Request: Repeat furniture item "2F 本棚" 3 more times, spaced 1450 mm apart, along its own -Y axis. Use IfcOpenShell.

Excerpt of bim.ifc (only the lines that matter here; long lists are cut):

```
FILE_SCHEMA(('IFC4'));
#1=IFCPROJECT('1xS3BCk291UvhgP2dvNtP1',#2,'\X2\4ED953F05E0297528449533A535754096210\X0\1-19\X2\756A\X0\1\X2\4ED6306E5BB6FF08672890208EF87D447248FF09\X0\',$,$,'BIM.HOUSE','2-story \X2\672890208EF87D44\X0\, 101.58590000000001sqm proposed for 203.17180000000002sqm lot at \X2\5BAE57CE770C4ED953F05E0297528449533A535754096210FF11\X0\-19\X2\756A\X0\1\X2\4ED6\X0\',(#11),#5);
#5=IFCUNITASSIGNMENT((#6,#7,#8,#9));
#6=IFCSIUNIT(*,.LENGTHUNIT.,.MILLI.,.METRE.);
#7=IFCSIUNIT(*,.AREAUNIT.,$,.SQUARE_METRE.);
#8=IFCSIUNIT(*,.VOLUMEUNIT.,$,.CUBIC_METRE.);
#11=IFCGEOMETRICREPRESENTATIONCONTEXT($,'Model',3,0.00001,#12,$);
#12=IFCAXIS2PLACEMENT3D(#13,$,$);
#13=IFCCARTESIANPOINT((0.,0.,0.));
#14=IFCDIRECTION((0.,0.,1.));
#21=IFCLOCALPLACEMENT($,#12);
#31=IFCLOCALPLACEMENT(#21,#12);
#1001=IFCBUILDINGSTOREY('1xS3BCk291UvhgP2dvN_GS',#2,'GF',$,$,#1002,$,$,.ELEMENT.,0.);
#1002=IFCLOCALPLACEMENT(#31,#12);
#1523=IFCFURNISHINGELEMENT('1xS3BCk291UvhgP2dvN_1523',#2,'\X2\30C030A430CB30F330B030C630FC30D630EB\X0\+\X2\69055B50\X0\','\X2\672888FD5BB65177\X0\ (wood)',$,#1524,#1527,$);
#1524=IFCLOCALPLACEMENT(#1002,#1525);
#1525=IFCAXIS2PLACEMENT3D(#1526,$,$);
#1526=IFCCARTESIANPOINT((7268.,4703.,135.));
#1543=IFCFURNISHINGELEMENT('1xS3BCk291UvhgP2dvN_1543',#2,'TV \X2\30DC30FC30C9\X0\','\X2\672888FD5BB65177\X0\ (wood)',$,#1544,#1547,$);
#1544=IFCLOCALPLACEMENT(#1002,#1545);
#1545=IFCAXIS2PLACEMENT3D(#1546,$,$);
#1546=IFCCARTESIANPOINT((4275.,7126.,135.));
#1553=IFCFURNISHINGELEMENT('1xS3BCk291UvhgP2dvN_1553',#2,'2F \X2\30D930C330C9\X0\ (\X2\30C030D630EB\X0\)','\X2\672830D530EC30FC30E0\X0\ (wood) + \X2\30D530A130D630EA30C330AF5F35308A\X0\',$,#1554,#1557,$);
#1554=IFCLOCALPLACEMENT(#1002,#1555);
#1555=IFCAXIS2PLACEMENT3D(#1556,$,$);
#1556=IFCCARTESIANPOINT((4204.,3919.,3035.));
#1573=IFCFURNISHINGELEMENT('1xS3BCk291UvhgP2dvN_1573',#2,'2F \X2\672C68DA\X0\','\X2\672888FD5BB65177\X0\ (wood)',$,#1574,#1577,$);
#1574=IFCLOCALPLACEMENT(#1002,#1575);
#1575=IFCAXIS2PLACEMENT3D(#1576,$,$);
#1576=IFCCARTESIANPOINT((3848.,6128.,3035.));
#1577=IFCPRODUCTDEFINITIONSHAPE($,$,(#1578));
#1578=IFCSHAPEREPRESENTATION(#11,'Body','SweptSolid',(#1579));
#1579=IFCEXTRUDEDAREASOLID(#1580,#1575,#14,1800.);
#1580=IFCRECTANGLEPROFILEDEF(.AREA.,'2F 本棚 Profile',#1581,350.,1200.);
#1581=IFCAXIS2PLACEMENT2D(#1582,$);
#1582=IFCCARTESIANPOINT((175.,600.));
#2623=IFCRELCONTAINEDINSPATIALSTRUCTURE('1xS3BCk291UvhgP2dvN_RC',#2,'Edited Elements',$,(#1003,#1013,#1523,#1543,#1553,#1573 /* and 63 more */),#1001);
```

```python
import ifcopenshell
import ifcopenshell.api.geometry
import ifcopenshell.api.root
import ifcopenshell.util.element
import ifcopenshell.util.placement

model = ifcopenshell.open("bim.ifc")


def reuse_history(source, copy):
    """copy_class also copies each property set's owner history, people and application; keep the originals."""
    for rel in copy.IsDefinedBy:
        if rel.is_a("IfcRelDefinesByProperties") and (history := rel.RelatingPropertyDefinition.OwnerHistory):
            rel.RelatingPropertyDefinition.OwnerHistory = source.OwnerHistory
            ifcopenshell.util.element.remove_deep2(model, history)


source = model.by_id(1573)
base = ifcopenshell.util.placement.get_local_placement(source.ObjectPlacement)
step = -base[:3, 1] * 1450.0

for i in range(1, 4):
    copy = ifcopenshell.api.root.copy_class(model, product=source)
    copy.Representation = ifcopenshell.util.element.copy_deep(
        model, source.Representation, exclude=["IfcGeometricRepresentationContext", "IfcRepresentationMap"]
    )
    reuse_history(source, copy)
    matrix = base.copy()
    matrix[:3, 3] += i * step
    print("added at", matrix[:3, 3].round(3) + 0.0)
    ifcopenshell.api.geometry.edit_object_placement(model, product=copy, matrix=matrix, is_si=False)

model.write("bim-out.ifc")
```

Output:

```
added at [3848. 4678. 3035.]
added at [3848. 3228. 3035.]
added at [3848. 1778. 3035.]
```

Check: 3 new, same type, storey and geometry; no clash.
